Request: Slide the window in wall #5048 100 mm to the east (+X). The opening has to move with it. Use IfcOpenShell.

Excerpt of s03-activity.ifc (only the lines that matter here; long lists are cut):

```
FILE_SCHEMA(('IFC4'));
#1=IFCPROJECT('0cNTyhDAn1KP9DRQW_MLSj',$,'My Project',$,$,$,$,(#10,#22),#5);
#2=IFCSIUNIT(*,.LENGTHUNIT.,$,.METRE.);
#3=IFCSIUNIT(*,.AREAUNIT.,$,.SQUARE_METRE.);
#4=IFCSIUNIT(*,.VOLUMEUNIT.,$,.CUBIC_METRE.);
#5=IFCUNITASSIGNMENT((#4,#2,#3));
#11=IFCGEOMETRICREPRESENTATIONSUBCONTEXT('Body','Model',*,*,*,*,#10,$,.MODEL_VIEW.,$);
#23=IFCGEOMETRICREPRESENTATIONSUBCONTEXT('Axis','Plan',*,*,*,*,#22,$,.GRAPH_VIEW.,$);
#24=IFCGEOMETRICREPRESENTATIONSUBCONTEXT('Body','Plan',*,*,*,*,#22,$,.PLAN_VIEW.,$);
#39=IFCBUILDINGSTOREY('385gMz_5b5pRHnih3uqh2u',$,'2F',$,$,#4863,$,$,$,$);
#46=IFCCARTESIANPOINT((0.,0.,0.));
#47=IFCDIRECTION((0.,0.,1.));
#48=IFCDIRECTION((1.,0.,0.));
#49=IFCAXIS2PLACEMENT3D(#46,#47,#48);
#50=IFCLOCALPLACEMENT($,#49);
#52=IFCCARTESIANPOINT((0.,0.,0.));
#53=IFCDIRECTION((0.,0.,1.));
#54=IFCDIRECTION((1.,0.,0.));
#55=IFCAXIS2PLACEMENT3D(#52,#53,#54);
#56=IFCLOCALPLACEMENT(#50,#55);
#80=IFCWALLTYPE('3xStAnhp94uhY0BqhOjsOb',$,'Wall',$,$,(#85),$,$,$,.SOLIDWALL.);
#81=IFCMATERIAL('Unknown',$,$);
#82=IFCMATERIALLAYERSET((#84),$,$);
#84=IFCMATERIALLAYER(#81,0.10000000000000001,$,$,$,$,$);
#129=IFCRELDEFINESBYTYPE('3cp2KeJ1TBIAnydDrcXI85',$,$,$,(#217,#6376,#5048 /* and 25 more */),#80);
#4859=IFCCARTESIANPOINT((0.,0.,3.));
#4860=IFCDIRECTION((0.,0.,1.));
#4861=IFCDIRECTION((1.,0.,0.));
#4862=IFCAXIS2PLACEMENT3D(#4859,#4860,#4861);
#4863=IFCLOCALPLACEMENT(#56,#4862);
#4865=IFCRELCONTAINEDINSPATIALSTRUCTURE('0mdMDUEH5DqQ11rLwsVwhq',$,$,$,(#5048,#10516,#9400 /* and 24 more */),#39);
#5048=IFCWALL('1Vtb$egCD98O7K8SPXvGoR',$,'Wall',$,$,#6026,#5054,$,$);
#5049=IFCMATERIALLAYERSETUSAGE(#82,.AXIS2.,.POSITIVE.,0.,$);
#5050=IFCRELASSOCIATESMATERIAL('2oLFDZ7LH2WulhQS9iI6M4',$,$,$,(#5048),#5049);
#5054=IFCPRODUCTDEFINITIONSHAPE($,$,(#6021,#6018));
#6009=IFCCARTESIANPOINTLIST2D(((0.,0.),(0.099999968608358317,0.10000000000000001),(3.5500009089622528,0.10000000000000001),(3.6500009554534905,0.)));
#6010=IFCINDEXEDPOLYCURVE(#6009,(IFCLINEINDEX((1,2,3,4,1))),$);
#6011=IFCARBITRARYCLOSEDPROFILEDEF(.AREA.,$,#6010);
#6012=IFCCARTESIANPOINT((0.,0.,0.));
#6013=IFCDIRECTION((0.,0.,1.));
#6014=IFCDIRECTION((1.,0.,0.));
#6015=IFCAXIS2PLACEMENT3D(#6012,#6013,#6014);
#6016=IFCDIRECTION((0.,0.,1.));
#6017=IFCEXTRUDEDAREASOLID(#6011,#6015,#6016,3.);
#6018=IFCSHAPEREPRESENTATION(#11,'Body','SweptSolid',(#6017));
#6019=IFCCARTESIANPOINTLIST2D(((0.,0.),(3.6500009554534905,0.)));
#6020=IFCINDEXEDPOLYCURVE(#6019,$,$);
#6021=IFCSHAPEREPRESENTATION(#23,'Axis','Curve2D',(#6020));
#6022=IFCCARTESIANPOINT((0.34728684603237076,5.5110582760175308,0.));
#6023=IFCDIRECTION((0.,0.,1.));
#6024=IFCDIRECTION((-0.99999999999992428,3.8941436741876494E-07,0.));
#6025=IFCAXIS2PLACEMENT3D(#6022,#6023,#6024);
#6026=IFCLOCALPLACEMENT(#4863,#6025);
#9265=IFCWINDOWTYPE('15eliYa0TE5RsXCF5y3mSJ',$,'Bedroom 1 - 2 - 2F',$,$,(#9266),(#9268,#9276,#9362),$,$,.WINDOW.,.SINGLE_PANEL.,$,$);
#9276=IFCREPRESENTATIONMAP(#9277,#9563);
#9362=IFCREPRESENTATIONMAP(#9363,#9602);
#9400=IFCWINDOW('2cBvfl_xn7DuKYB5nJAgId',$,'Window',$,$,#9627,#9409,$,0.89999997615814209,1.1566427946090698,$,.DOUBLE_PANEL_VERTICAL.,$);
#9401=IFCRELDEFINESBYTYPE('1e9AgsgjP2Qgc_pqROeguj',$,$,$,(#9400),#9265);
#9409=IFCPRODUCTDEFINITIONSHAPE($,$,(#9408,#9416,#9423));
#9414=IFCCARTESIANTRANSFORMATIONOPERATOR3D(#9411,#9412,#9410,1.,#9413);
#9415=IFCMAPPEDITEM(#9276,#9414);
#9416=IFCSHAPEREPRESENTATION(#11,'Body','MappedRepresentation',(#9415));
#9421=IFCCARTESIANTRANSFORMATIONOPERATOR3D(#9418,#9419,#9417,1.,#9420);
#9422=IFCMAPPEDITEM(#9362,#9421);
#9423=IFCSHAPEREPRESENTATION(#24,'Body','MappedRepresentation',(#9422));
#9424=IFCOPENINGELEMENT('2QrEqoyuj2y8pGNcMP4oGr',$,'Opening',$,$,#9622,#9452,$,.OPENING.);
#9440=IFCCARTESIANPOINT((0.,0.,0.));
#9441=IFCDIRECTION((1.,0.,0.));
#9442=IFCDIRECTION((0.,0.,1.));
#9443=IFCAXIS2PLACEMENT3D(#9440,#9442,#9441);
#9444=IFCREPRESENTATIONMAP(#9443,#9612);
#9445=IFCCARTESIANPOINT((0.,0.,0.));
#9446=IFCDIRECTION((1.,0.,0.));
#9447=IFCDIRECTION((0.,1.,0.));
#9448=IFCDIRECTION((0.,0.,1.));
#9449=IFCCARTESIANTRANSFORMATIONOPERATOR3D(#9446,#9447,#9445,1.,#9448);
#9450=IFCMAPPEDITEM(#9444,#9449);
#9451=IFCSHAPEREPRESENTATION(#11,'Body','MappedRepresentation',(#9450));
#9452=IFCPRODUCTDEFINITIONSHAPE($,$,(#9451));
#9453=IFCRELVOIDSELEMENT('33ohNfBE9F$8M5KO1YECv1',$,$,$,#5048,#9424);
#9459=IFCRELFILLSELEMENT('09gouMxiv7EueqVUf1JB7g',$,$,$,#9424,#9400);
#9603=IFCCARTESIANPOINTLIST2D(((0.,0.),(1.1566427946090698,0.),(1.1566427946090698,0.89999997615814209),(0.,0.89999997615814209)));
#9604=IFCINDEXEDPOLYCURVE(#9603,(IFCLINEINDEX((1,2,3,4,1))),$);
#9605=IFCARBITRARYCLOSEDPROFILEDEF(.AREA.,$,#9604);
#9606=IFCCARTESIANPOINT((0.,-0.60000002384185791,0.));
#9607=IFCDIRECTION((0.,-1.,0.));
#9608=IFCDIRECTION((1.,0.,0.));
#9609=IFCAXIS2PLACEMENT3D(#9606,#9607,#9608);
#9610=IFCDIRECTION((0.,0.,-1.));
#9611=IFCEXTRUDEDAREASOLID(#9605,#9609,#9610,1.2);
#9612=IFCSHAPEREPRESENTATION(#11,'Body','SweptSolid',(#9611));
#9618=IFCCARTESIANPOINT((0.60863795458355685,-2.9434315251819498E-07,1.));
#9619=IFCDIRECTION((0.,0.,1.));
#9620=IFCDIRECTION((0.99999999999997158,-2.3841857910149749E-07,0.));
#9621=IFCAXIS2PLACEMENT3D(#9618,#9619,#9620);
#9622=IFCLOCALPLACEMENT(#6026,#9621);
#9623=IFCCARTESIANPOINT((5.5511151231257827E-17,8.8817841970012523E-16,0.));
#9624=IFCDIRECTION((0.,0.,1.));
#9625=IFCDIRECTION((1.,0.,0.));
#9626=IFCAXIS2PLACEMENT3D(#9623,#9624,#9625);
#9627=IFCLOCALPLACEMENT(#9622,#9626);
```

```python
import ifcopenshell
import ifcopenshell.api.geometry
import ifcopenshell.util.placement
import ifcopenshell.util.unit

model = ifcopenshell.open("s03-activity.ifc")
unit_scale = ifcopenshell.util.unit.calculate_unit_scale(model)

window = model.by_id(9400)
opening = window.FillsVoids[0].RelatingOpeningElement
wall = opening.VoidsElements[0].RelatingBuildingElement

wall_matrix = ifcopenshell.util.placement.get_local_placement(wall.ObjectPlacement)
shift = wall_matrix[:3, 0] * -0.1 / unit_scale
before = ifcopenshell.util.placement.get_local_placement(window.ObjectPlacement)[:3, 3].copy()

# The window is placed relative to its opening, so it follows when the opening moves.
matrix = ifcopenshell.util.placement.get_local_placement(opening.ObjectPlacement)
matrix[:3, 3] += shift
ifcopenshell.api.geometry.edit_object_placement(
    model, product=opening, matrix=matrix, is_si=False, should_transform_children=True
)

after = ifcopenshell.util.placement.get_local_placement(window.ObjectPlacement)[:3, 3]
print("window moved by", (after - before).round(3) + 0.0)

model.write("s03-activity_edited.ifc")
```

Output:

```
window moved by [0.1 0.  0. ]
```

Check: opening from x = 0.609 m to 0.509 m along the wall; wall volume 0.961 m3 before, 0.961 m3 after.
